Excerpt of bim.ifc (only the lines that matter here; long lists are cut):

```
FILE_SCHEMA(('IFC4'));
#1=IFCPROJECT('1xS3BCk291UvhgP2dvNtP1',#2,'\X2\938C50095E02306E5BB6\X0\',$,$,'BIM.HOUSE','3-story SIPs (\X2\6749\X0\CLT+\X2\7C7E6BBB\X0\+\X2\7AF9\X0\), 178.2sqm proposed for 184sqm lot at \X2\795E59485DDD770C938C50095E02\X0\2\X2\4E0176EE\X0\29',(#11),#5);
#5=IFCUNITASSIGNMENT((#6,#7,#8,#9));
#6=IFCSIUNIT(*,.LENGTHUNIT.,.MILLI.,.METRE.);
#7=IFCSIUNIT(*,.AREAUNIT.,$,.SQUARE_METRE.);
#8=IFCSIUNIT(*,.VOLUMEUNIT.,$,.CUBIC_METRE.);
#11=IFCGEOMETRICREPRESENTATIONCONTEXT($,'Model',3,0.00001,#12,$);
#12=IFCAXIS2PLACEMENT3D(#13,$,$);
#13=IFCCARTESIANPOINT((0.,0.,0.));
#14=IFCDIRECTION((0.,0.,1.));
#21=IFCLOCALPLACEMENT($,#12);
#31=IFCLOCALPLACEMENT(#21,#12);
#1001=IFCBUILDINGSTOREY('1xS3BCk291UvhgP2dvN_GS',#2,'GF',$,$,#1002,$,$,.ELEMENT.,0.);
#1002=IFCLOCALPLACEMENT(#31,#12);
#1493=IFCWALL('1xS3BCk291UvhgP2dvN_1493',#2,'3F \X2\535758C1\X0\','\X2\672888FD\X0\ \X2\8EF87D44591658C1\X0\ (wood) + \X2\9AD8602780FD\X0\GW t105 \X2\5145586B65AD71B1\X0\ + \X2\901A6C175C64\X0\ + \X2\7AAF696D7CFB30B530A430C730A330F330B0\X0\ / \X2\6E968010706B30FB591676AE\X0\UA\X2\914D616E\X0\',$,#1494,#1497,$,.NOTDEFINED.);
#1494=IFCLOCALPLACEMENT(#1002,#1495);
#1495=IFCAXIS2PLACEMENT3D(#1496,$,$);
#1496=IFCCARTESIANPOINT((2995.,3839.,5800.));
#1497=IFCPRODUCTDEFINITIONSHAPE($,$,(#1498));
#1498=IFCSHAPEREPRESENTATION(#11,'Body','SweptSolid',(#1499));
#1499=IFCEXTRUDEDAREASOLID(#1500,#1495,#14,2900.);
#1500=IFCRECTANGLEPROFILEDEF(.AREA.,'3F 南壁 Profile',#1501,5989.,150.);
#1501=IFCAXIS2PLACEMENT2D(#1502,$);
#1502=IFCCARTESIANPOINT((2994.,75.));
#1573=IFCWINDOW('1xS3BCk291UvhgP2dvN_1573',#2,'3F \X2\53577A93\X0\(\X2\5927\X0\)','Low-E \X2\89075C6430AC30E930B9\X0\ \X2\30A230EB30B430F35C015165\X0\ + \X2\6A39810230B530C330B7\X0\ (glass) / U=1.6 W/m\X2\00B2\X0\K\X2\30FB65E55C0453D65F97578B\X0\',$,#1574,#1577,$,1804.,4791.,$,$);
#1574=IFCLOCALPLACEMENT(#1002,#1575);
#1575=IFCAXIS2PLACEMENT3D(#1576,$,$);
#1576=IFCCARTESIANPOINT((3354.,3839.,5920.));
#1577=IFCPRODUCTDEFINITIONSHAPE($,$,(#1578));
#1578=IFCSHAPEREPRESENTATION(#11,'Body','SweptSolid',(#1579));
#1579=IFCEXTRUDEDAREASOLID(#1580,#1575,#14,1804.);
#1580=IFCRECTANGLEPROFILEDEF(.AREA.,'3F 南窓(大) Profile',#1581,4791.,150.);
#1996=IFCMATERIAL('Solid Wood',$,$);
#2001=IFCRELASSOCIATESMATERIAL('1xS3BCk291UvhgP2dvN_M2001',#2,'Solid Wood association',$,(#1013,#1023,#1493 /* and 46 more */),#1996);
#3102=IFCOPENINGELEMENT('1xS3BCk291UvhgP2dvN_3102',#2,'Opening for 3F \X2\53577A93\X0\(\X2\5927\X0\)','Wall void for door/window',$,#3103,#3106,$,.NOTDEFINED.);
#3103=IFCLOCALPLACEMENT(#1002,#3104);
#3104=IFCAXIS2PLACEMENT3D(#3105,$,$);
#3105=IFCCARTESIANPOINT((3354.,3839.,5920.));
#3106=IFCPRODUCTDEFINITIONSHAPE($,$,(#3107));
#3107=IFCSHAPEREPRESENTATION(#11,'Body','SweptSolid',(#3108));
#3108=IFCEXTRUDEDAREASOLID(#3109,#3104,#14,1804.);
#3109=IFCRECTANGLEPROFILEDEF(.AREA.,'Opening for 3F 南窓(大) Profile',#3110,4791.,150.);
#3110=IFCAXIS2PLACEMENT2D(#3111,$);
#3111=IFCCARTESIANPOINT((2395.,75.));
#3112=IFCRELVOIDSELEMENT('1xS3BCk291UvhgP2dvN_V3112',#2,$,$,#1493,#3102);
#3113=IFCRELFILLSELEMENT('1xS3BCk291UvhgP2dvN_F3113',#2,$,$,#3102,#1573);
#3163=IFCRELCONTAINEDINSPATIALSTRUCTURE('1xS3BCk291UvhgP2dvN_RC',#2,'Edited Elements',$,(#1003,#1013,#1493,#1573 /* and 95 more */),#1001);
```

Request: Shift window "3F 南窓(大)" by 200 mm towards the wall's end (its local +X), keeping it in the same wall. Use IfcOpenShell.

```python
import ifcopenshell
import ifcopenshell.api.geometry
import ifcopenshell.util.placement

model = ifcopenshell.open("bim.ifc")

window = model.by_guid("1xS3BCk291UvhgP2dvN_1573")
opening = window.FillsVoids[0].RelatingOpeningElement
wall = opening.VoidsElements[0].RelatingBuildingElement

wall_matrix = ifcopenshell.util.placement.get_local_placement(wall.ObjectPlacement)
shift = wall_matrix[:3, 0] * 200.0
before = ifcopenshell.util.placement.get_local_placement(window.ObjectPlacement)[:3, 3].copy()

# The window is not placed relative to its opening, so move both.
for product in (opening, window):
    matrix = ifcopenshell.util.placement.get_local_placement(product.ObjectPlacement)
    matrix[:3, 3] += shift
    ifcopenshell.api.geometry.edit_object_placement(model, product=product, matrix=matrix, is_si=False)

after = ifcopenshell.util.placement.get_local_placement(window.ObjectPlacement)[:3, 3]
print("window moved by", (after - before).round(3) + 0.0)

model.write("bim_updated.ifc")
```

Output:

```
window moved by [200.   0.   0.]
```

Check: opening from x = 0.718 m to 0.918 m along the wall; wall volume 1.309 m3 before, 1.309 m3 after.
